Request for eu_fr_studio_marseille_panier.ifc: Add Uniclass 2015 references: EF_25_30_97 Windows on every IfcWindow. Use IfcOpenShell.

First a look at what the model holds.

```python
import ifcopenshell

model = ifcopenshell.open("eu_fr_studio_marseille_panier.ifc")
print(model.schema)
print("classifications:", [c.Name for c in model.by_type("IfcClassification")])
for ifc_class in ("IfcDoor", "IfcRoof", "IfcStair", "IfcWall", "IfcWindow"):
    print(ifc_class, len(model.by_type(ifc_class)))
```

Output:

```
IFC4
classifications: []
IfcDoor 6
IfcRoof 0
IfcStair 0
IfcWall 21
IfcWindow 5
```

```python
import ifcopenshell
import ifcopenshell.api.classification

model = ifcopenshell.open("eu_fr_studio_marseille_panier.ifc")

system = ifcopenshell.api.classification.add_classification(model, classification="Uniclass 2015")

codes = {
    "IfcWindow": ("EF_25_30_97", "Windows"),
}
for ifc_class, (code, name) in codes.items():
    products = model.by_type(ifc_class)
    ifcopenshell.api.classification.add_reference(
        model, products=products, classification=system, identification=code, name=name
    )
    print(code, len(products))

model.write("eu_fr_studio_marseille_panier_v2.ifc")
```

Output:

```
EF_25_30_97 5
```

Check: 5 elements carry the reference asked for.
